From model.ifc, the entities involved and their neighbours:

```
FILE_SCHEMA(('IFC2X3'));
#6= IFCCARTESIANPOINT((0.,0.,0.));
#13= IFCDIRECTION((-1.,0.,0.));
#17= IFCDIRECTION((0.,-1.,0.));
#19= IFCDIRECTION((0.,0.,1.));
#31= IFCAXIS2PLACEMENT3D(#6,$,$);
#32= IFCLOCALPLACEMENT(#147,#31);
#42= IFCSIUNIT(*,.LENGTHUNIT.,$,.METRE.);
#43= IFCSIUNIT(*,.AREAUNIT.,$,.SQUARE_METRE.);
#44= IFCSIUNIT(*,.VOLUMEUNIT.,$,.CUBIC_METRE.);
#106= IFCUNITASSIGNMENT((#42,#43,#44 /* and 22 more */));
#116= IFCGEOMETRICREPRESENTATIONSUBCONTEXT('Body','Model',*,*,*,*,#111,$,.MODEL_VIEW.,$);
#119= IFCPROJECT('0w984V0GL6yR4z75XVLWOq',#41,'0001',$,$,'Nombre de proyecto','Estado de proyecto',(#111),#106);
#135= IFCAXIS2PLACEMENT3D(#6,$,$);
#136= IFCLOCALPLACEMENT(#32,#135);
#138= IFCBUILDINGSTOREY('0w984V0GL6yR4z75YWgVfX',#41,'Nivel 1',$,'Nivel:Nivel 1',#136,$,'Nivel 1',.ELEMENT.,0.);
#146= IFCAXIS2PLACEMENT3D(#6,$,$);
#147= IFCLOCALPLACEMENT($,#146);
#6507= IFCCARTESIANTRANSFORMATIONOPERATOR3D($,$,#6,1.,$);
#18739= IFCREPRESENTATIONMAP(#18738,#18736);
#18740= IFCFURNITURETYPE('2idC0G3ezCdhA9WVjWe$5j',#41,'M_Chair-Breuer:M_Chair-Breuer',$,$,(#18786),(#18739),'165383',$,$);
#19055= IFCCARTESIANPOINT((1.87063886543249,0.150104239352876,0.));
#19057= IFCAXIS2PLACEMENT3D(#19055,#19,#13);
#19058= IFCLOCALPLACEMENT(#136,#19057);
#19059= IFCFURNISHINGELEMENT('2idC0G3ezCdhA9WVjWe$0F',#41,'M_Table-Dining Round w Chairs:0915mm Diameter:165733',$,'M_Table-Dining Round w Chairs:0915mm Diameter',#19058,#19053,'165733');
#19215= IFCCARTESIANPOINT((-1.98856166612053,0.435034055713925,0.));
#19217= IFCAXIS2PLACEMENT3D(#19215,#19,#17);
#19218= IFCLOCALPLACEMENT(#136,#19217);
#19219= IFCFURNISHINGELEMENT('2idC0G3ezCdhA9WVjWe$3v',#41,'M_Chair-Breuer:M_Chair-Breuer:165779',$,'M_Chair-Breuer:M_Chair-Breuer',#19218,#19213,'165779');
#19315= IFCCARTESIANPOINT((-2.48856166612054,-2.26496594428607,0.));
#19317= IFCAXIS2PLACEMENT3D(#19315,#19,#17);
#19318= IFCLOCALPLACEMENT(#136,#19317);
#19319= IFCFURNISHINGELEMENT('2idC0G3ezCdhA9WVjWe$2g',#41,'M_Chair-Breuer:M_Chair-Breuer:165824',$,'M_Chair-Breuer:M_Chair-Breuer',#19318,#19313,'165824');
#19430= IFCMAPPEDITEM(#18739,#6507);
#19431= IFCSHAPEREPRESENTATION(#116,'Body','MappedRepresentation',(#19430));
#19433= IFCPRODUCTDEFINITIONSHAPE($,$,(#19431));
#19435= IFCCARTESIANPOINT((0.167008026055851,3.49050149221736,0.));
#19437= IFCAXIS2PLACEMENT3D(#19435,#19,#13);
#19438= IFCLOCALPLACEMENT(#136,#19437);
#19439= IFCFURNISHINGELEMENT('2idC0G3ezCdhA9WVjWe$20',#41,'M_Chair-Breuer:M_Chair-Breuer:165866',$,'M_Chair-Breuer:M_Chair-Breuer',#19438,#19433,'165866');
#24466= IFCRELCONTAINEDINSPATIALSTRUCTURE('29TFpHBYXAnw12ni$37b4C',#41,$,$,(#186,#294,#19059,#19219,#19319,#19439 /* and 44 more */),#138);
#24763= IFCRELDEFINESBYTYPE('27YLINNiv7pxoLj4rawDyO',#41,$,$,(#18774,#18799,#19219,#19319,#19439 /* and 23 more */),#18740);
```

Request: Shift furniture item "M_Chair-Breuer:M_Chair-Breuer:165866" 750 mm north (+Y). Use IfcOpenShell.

```python
import ifcopenshell
import ifcopenshell.api.geometry
import ifcopenshell.util.placement
import ifcopenshell.util.unit

model = ifcopenshell.open("model.ifc")
unit_scale = ifcopenshell.util.unit.calculate_unit_scale(model)

item = model.by_guid("2idC0G3ezCdhA9WVjWe$20")
matrix = ifcopenshell.util.placement.get_local_placement(item.ObjectPlacement)
matrix[1, 3] += 0.75 / unit_scale
ifcopenshell.api.geometry.edit_object_placement(model, product=item, matrix=matrix, is_si=False)

print(ifcopenshell.util.placement.get_local_placement(item.ObjectPlacement).round(3) + 0.0)

model.write("model_updated.ifc")
```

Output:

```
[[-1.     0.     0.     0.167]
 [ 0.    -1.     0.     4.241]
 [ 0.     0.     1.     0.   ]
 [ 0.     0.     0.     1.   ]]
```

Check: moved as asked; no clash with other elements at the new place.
